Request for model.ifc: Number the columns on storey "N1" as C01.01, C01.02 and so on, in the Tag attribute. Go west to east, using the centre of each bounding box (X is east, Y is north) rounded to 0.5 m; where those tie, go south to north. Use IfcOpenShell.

First a look at what the model holds.

```python
import ifcopenshell
import ifcopenshell.util.element
import ifcopenshell.util.placement

model = ifcopenshell.open("model.ifc")
print(model.schema)
storey = next(s for s in model.by_type("IfcBuildingStorey") if s.Name == "N1")
columns = [e for e in ifcopenshell.util.element.get_decomposition(storey) if e.is_a("IfcColumn")]
for e in sorted(columns, key=lambda e: e.id()):
    origin = ifcopenshell.util.placement.get_local_placement(e.ObjectPlacement)[:3, 3]
    print(e.id(), e.Tag, e.Name, origin.round(2) + 0.0, sep=" | ")
```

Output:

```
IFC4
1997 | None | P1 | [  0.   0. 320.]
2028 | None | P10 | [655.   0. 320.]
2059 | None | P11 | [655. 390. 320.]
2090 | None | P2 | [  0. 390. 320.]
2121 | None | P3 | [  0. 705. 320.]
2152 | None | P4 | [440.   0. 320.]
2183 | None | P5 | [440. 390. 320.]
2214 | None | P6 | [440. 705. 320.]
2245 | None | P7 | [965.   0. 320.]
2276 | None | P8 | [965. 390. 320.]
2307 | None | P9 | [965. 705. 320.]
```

```python
import ifcopenshell
import ifcopenshell.geom
import ifcopenshell.util.element
import ifcopenshell.util.shape

model = ifcopenshell.open("model.ifc")
settings = ifcopenshell.geom.settings()
settings.set("use-world-coords", True)


def centre(element):
    shape = ifcopenshell.geom.create_shape(settings, element)
    return ifcopenshell.util.shape.get_bbox_centroid(shape.geometry)


storey = next(s for s in model.by_type("IfcBuildingStorey") if s.Name == "N1")
columns = [e for e in ifcopenshell.util.element.get_decomposition(storey) if e.is_a("IfcColumn")]

# Insertion points can sit at a corner or the storey origin, so sort by the geometry (in metres).
centres = {e: centre(e) for e in columns}
columns.sort(key=lambda e: (round(centres[e][0] / 0.5), centres[e][1]))

for i, e in enumerate(columns, start=1):
    number = f"C01.{i:02d}"
    e.Tag = number
    print(e.id(), number)

model.write("model-out.ifc")
```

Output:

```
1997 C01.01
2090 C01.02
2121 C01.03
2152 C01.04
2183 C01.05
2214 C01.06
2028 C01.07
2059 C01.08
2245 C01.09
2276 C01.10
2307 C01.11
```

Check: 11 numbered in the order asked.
